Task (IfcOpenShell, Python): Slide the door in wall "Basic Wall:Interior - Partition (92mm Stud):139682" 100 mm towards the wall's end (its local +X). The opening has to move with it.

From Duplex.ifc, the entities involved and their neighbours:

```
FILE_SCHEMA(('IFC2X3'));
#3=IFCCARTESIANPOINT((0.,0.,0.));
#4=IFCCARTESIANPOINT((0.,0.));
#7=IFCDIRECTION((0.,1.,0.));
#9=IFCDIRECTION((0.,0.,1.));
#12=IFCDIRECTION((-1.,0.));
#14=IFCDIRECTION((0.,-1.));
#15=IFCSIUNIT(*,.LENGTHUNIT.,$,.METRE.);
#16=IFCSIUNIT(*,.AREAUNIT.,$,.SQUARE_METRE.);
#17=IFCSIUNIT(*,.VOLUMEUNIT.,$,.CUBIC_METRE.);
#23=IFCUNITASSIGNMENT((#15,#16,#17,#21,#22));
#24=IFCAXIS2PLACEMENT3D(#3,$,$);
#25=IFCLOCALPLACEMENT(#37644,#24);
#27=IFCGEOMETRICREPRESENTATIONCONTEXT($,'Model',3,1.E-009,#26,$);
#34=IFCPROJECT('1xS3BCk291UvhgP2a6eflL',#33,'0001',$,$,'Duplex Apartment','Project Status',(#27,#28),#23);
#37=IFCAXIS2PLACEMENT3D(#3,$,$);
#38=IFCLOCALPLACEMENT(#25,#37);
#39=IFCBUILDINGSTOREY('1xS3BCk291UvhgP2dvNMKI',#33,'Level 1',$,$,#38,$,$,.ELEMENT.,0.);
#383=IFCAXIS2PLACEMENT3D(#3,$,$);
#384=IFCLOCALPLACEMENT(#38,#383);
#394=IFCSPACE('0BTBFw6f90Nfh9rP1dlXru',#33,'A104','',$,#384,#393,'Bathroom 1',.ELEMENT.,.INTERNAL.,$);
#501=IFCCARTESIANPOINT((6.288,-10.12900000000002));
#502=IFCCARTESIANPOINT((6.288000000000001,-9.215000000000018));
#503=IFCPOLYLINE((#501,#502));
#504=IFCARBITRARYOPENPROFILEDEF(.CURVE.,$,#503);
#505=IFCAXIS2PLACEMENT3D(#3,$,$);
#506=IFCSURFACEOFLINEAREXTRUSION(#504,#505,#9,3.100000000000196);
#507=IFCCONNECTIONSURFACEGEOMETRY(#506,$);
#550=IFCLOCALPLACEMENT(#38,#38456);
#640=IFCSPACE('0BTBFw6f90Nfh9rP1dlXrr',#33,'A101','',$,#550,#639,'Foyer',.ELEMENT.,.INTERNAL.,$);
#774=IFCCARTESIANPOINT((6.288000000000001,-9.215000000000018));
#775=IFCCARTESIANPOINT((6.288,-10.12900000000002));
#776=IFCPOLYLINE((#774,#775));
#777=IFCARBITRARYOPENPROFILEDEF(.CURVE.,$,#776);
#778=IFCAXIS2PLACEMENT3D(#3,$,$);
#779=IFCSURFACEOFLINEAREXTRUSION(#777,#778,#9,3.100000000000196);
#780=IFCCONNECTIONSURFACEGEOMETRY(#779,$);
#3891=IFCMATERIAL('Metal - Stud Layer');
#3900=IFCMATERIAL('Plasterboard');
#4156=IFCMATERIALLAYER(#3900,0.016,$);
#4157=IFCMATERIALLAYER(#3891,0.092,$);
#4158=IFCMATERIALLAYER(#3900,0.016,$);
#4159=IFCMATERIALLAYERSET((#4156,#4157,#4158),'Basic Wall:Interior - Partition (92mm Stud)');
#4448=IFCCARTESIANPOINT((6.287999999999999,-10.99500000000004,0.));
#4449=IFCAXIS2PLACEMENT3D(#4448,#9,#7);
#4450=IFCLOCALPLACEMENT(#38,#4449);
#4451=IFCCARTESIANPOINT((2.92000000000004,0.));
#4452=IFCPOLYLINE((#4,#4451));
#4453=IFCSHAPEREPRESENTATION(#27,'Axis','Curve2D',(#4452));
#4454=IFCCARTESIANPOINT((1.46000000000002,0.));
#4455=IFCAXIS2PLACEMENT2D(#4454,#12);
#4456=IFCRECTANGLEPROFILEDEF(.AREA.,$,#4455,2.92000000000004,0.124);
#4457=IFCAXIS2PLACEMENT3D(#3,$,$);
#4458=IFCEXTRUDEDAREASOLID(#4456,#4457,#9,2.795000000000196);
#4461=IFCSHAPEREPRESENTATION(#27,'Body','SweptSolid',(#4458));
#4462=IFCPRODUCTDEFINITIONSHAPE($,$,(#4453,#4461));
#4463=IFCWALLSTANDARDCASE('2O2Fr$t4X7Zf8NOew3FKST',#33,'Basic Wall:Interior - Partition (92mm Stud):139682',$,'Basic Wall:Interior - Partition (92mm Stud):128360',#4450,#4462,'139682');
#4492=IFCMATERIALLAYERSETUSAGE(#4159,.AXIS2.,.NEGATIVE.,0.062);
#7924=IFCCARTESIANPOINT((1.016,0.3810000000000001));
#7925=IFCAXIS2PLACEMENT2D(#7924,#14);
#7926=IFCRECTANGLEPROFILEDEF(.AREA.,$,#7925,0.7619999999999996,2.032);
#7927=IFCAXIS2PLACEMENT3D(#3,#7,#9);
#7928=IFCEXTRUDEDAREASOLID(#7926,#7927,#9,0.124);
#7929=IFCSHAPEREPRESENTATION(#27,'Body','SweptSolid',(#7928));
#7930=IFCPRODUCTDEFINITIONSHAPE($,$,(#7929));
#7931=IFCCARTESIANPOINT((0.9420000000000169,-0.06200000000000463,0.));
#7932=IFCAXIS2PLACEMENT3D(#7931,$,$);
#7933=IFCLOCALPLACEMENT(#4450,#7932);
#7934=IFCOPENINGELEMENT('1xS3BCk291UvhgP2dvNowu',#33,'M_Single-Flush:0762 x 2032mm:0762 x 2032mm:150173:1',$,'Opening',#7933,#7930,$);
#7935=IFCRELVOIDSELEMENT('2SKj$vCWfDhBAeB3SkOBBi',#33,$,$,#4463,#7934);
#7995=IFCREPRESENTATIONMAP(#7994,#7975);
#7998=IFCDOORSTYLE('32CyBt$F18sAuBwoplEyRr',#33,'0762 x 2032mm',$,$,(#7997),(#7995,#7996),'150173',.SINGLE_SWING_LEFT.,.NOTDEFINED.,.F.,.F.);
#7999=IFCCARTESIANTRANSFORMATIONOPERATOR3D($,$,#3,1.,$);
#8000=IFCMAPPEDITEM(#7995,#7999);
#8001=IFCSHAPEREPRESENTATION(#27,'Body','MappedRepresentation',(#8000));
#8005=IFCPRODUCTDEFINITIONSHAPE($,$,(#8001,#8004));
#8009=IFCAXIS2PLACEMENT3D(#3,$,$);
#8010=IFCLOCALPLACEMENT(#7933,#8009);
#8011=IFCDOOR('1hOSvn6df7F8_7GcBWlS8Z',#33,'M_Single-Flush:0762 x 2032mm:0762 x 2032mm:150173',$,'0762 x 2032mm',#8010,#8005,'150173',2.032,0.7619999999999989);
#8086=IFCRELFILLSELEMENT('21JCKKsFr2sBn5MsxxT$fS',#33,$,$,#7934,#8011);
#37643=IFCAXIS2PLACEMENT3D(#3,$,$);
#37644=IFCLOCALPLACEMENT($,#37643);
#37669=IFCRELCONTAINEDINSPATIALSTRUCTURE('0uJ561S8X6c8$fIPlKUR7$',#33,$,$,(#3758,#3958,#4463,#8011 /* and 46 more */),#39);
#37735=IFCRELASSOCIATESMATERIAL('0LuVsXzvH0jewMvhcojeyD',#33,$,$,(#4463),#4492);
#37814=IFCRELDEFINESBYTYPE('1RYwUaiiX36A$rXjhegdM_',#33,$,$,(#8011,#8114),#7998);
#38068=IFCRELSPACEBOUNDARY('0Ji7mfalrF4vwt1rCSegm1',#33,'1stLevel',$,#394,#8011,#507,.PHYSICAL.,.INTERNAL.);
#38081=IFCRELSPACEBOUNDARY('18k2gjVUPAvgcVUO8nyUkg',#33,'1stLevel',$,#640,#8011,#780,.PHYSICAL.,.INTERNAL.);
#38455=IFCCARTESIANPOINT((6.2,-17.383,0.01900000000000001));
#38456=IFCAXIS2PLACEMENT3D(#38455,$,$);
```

```python
import numpy as np
import ifcopenshell
import ifcopenshell.api.geometry
import ifcopenshell.util.placement

model = ifcopenshell.open("Duplex.ifc")

door = model.by_guid("1hOSvn6df7F8_7GcBWlS8Z")
opening = door.FillsVoids[0].RelatingOpeningElement
wall = opening.VoidsElements[0].RelatingBuildingElement

wall_matrix = ifcopenshell.util.placement.get_local_placement(wall.ObjectPlacement)
shift = wall_matrix[:3, 0] * 0.1
before = ifcopenshell.util.placement.get_local_placement(door.ObjectPlacement)[:3, 3].copy()

# The door is placed relative to its opening, so it follows when the opening moves.
matrix = ifcopenshell.util.placement.get_local_placement(opening.ObjectPlacement)
matrix[:3, 3] += shift
ifcopenshell.api.geometry.edit_object_placement(
    model, product=opening, matrix=matrix, is_si=False, should_transform_children=True
)

# Space boundary surfaces are stored in each space's coordinates; move them too.
for rel in door.ProvidesBoundaries:
    if not rel.ConnectionGeometry:
        continue
    surface = rel.ConnectionGeometry.SurfaceOnRelatingElement
    space_matrix = ifcopenshell.util.placement.get_local_placement(rel.RelatingSpace.ObjectPlacement)
    point = np.array(surface.Position.Location.Coordinates) + space_matrix[:3, :3].T @ shift
    surface.Position = model.createIfcAxis2Placement3D(
        model.createIfcCartesianPoint(point.tolist()), surface.Position.Axis, surface.Position.RefDirection
    )

after = ifcopenshell.util.placement.get_local_placement(door.ObjectPlacement)[:3, 3]
print("door moved by", (after - before).round(3) + 0.0)

model.write("Duplex_edited.ifc")
```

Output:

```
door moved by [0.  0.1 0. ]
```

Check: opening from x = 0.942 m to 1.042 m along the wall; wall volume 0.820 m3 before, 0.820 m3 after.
